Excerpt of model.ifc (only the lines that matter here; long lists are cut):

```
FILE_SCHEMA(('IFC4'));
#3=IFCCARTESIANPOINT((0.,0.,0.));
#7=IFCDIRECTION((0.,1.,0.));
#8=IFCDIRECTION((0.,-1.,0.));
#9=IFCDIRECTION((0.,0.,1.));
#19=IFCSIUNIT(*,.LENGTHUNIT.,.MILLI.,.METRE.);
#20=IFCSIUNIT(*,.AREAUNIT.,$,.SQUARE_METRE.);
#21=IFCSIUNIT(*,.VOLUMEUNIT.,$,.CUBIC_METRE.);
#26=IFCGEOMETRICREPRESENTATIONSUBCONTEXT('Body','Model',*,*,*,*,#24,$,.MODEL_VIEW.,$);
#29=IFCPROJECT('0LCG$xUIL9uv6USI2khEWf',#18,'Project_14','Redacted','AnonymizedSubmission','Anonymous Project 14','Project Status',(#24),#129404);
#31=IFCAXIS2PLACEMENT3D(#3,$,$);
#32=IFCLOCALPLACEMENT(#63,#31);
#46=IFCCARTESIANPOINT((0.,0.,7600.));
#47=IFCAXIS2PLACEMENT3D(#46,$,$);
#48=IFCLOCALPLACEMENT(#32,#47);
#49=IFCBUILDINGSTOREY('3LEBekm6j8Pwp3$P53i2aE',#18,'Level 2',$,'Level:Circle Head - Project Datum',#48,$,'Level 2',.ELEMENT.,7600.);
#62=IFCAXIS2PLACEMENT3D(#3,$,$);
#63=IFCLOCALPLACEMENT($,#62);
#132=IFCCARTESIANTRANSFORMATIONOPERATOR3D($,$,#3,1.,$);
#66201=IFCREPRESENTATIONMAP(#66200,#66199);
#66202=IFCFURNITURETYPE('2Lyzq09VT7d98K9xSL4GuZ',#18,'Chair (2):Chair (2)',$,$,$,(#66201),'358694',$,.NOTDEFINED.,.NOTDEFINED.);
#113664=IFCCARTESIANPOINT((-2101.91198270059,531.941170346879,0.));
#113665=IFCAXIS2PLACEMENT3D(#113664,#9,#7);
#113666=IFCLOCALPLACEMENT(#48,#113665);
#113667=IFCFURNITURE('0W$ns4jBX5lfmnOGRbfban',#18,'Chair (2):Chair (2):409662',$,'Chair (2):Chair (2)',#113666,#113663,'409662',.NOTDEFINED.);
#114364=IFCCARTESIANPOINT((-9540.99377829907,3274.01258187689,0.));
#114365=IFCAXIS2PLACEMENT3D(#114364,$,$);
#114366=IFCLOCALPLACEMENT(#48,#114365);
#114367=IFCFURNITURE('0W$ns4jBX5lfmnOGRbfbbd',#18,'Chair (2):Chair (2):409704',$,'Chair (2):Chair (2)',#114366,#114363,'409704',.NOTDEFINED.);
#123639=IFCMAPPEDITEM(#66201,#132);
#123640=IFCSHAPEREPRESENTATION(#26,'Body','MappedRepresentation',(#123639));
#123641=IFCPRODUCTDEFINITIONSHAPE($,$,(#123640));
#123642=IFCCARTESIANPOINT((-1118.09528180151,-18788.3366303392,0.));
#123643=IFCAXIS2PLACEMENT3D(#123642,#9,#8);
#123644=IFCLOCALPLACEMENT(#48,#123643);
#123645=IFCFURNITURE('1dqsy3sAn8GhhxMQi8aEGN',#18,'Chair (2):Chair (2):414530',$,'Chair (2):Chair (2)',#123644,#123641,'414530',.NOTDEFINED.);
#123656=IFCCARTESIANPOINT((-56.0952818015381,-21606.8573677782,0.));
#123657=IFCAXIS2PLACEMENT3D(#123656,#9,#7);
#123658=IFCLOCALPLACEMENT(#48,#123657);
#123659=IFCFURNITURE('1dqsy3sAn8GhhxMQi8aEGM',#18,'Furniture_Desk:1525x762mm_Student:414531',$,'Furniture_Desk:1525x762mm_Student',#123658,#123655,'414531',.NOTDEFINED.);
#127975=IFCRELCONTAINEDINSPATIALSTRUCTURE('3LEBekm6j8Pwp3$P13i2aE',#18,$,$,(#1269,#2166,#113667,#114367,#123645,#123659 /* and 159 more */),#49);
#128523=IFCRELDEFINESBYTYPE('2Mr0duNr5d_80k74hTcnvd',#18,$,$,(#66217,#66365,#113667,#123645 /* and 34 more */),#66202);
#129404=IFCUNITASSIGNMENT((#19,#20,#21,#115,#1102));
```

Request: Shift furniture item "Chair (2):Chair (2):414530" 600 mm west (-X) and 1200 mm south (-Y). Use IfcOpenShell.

```python
import ifcopenshell
import ifcopenshell.api.geometry
import ifcopenshell.util.placement

model = ifcopenshell.open("model.ifc")

item = model.by_guid("1dqsy3sAn8GhhxMQi8aEGN")
matrix = ifcopenshell.util.placement.get_local_placement(item.ObjectPlacement)
matrix[0, 3] -= 600.0
matrix[1, 3] -= 1200.0
ifcopenshell.api.geometry.edit_object_placement(model, product=item, matrix=matrix, is_si=False)

print(ifcopenshell.util.placement.get_local_placement(item.ObjectPlacement).round(3) + 0.0)

model.write("model_edited.ifc")
```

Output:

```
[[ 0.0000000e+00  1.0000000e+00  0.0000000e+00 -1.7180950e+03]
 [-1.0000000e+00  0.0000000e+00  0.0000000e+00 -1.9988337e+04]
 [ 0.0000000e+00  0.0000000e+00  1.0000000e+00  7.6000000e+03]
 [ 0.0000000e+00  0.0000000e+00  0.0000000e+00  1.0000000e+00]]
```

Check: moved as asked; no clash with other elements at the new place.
